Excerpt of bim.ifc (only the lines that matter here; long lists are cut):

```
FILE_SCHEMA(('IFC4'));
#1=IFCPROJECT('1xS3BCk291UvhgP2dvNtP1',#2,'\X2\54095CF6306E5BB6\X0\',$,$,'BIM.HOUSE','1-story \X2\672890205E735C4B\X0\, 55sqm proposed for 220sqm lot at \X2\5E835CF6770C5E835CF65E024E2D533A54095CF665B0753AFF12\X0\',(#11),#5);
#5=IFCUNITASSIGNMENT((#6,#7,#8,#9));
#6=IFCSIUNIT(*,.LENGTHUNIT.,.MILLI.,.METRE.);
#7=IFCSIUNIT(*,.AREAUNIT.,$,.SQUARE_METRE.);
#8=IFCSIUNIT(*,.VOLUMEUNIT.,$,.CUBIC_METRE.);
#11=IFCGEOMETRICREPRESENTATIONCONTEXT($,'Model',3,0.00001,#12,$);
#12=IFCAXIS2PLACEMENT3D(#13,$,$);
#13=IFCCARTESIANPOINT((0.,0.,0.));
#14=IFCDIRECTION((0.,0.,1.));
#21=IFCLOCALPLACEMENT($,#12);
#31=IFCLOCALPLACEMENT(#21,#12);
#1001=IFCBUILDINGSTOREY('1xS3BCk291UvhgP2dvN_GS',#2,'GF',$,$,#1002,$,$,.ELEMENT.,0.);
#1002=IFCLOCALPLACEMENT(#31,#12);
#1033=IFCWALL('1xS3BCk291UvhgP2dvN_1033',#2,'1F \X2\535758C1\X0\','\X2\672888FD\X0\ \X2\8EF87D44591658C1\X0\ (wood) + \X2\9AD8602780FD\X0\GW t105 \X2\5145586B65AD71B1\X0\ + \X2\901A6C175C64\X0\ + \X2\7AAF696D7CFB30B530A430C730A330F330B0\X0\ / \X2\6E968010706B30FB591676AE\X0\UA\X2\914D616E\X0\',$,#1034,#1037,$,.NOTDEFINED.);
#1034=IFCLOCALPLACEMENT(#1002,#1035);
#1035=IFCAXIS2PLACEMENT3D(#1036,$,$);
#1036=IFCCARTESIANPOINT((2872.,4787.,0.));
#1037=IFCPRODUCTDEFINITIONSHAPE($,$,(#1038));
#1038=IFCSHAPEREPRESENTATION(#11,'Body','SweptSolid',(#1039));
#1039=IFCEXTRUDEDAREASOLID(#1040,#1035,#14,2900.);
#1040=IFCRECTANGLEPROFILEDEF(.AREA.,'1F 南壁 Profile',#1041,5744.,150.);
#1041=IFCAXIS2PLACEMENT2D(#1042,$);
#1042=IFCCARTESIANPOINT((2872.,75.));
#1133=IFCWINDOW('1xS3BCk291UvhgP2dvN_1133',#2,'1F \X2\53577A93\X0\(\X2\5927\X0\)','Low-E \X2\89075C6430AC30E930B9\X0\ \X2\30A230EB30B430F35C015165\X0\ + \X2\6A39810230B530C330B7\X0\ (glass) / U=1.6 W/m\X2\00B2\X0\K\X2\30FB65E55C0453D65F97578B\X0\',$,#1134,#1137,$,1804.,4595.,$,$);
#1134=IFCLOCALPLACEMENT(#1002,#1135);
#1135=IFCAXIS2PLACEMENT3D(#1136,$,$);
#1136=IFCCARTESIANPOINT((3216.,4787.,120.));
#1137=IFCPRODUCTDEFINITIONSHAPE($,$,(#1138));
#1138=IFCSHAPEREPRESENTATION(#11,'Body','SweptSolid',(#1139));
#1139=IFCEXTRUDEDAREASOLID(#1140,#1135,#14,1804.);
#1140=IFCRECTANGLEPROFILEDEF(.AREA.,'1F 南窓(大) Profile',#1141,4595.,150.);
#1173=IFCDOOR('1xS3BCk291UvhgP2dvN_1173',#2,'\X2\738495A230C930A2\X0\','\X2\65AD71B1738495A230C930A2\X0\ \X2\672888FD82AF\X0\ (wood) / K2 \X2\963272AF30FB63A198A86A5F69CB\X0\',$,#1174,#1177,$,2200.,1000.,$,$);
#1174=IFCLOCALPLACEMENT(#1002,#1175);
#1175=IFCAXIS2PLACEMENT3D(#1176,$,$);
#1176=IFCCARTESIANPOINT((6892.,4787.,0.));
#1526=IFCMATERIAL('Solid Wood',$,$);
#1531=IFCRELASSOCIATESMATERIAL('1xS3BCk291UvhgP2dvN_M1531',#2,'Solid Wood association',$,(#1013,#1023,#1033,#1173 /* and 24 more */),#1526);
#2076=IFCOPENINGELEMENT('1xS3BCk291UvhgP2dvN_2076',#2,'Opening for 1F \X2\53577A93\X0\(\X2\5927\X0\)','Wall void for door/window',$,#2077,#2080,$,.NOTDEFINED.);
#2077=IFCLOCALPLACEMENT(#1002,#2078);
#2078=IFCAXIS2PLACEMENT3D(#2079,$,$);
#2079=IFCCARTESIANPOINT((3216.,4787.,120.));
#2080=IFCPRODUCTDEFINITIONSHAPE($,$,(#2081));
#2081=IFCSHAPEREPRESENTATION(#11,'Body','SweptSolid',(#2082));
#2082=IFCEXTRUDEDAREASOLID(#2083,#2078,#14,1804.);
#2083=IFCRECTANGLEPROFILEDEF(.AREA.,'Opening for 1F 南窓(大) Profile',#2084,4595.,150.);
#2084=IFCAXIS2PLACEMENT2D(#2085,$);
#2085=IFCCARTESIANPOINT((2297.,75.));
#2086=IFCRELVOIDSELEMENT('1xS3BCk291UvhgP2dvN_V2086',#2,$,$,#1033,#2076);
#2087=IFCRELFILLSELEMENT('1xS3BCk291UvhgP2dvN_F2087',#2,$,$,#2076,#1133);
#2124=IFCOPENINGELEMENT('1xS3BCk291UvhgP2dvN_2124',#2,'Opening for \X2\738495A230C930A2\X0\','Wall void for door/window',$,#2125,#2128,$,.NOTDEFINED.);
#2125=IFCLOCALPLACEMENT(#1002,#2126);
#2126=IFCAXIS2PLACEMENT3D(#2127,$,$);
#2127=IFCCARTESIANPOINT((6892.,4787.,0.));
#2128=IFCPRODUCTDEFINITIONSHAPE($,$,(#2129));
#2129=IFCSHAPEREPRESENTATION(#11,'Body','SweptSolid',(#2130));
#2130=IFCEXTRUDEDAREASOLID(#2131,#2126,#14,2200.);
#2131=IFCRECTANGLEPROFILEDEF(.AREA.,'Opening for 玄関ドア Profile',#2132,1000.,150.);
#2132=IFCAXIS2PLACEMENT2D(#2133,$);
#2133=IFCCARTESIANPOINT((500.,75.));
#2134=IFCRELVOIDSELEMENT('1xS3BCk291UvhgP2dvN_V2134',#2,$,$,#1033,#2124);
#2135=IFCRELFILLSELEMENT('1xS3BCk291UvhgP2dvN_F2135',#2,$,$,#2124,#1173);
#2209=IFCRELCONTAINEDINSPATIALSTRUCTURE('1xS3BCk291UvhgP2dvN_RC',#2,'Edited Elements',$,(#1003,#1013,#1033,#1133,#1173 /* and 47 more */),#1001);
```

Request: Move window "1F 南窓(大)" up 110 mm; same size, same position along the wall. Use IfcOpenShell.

```python
import numpy as np
import ifcopenshell
import ifcopenshell.api.geometry
import ifcopenshell.util.placement
import ifcopenshell.util.unit

model = ifcopenshell.open("bim.ifc")
unit_scale = ifcopenshell.util.unit.calculate_unit_scale(model)

window = model.by_guid("1xS3BCk291UvhgP2dvN_1133")
opening = window.FillsVoids[0].RelatingOpeningElement
dz = 110.0

shift = np.array([0.0, 0.0, dz])
# The window is not placed relative to its opening, so move both.
for product in (opening, window):
    matrix = ifcopenshell.util.placement.get_local_placement(product.ObjectPlacement)
    matrix[:3, 3] += shift
    ifcopenshell.api.geometry.edit_object_placement(model, product=product, matrix=matrix, is_si=False)

print(f"moved by {dz * unit_scale:+.3f} m")

model.write("bim-out.ifc")
```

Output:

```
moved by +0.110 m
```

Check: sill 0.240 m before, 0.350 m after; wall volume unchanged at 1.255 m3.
